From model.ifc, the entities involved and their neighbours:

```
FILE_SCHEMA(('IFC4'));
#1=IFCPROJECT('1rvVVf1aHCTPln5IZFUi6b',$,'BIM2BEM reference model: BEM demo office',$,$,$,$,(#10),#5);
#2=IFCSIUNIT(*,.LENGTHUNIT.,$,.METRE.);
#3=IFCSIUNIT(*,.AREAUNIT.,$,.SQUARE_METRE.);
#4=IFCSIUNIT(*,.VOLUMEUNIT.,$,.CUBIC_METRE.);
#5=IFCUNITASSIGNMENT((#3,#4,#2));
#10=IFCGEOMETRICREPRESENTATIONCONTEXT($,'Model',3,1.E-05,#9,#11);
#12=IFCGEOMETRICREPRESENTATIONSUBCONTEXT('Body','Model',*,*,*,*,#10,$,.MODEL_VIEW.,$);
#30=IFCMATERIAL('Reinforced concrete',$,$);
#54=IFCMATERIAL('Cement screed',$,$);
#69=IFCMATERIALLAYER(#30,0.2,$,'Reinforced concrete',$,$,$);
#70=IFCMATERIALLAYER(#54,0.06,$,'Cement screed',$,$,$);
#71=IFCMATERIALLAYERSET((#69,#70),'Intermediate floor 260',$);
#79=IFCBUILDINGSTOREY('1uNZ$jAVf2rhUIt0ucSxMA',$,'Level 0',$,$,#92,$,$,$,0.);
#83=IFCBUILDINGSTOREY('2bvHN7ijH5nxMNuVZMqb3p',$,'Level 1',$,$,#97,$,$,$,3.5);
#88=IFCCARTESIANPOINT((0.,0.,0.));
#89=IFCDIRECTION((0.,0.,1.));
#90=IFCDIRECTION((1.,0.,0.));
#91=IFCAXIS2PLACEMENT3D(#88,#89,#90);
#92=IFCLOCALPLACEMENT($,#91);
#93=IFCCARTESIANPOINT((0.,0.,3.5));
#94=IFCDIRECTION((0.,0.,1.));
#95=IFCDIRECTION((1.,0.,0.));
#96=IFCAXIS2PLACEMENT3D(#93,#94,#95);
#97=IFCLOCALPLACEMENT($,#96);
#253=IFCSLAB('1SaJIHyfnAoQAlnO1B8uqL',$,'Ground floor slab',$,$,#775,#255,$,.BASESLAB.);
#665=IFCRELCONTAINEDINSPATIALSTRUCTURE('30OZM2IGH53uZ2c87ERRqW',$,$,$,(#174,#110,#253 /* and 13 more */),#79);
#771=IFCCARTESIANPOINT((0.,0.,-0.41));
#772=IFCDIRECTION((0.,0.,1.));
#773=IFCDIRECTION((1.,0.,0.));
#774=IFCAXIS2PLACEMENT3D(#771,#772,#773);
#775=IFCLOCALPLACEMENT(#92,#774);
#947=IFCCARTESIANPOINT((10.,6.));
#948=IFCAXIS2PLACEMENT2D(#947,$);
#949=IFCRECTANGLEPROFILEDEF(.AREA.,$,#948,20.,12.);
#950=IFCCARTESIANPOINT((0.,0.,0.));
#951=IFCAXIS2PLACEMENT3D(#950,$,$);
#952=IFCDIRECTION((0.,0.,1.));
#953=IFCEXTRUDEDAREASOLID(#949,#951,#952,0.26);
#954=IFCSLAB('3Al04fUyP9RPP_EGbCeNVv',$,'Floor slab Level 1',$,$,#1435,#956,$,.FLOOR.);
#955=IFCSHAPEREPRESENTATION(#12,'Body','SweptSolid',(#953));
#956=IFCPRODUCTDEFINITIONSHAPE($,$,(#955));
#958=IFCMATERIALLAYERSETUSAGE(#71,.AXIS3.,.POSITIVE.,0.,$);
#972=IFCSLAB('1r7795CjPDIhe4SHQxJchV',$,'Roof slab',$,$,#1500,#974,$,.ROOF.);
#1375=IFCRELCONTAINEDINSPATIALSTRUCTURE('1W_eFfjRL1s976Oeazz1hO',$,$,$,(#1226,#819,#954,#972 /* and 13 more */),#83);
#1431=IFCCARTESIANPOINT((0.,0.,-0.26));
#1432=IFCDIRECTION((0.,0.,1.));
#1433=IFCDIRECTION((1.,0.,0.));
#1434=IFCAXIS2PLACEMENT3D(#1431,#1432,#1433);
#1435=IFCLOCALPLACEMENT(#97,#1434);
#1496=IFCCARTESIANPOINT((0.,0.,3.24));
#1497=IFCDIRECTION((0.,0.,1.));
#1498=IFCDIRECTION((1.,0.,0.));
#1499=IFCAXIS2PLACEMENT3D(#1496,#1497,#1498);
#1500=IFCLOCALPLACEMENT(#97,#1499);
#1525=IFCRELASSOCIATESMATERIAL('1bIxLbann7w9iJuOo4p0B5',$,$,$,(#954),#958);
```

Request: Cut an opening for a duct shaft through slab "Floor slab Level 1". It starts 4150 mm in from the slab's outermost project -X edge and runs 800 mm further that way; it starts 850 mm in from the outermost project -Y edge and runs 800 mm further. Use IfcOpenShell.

```python
import numpy as np
import ifcopenshell
import ifcopenshell.api.feature
import ifcopenshell.api.geometry
import ifcopenshell.api.root
import ifcopenshell.geom
import ifcopenshell.util.placement
import ifcopenshell.util.representation
import ifcopenshell.util.shape
import ifcopenshell.util.unit

model = ifcopenshell.open("model.ifc")
unit_scale = ifcopenshell.util.unit.calculate_unit_scale(model)
settings = ifcopenshell.geom.settings()


def volume(element):
    """Net volume in cubic metres, openings subtracted."""
    shape = ifcopenshell.geom.create_shape(settings, element)
    return ifcopenshell.util.shape.get_volume(shape.geometry)


slab = model.by_guid("3Al04fUyP9RPP_EGbCeNVv")
before = volume(slab)

# Extent in the slab's own axes, in metres. The edges named are its -X and -Y sides.
slab_shape = ifcopenshell.geom.create_shape(settings, slab)
vertices = ifcopenshell.util.shape.get_vertices(slab_shape.geometry)
x_min, y_min, bottom = vertices.min(axis=0)
top = vertices[:, 2].max()

opening = ifcopenshell.api.root.create_entity(model, ifc_class="IfcOpeningElement", name="Duct shaft opening", predefined_type="OPENING")
context = ifcopenshell.util.representation.get_context(model, "Model", "Body", "MODEL_VIEW")
width, depth = 0.8, 0.8
outline = [(0.0, 0.0), (width, 0.0), (width, depth), (0.0, depth), (0.0, 0.0)]
# Overshoot both faces by 50 mm so the cut is clean.
shape = ifcopenshell.api.geometry.add_slab_representation(
    model, context=context, depth=top - bottom + 0.1, polyline=outline
)
ifcopenshell.api.geometry.assign_representation(model, product=opening, representation=shape)

matrix = ifcopenshell.util.placement.get_local_placement(slab.ObjectPlacement)
matrix[:, 3] = matrix @ np.append(np.array([x_min + 4.15, y_min + 0.85, bottom - 0.05]) / unit_scale, 1.0)
ifcopenshell.api.geometry.edit_object_placement(model, product=opening, matrix=matrix, is_si=False)
ifcopenshell.api.feature.add_feature(model, feature=opening, element=slab)

after = volume(slab)

print(f"slab volume {before:.3f} -> {after:.3f} m3")

model.write("model_updated.ifc")
```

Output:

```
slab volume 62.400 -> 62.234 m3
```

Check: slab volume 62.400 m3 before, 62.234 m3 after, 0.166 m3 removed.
